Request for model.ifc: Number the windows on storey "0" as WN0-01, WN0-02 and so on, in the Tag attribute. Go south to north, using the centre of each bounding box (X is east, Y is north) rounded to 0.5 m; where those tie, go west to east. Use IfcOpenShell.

First a look at what the model holds.

```python
import ifcopenshell
import ifcopenshell.util.element
import ifcopenshell.util.placement

model = ifcopenshell.open("model.ifc")
print(model.schema)
storey = next(s for s in model.by_type("IfcBuildingStorey") if s.Name == "0")
windows = [e for e in ifcopenshell.util.element.get_decomposition(storey) if e.is_a("IfcWindow")]
for e in sorted(windows, key=lambda e: e.id()):
    origin = ifcopenshell.util.placement.get_local_placement(e.ObjectPlacement)[:3, 3]
    print(e.id(), e.Tag, e.Name, origin.round(2) + 0.0, sep=" | ")
```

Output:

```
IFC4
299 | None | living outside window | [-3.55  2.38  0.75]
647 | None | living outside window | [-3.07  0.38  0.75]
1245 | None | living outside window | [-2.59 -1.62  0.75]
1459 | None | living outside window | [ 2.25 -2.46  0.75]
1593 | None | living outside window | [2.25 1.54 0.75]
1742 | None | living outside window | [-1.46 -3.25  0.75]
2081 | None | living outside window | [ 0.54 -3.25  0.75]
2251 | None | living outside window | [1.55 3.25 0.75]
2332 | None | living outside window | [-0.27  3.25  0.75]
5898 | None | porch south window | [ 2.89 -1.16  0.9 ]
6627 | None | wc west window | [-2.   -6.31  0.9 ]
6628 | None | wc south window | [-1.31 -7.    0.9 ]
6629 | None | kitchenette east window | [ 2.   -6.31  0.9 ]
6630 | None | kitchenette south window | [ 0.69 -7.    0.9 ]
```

```python
import ifcopenshell
import ifcopenshell.geom
import ifcopenshell.util.element
import ifcopenshell.util.shape

model = ifcopenshell.open("model.ifc")
settings = ifcopenshell.geom.settings()
settings.set("use-world-coords", True)


def centre(element):
    shape = ifcopenshell.geom.create_shape(settings, element)
    return ifcopenshell.util.shape.get_bbox_centroid(shape.geometry)


storey = next(s for s in model.by_type("IfcBuildingStorey") if s.Name == "0")
windows = [e for e in ifcopenshell.util.element.get_decomposition(storey) if e.is_a("IfcWindow")]

# Insertion points can sit at a corner or the storey origin, so sort by the geometry (in metres).
centres = {e: centre(e) for e in windows}
windows.sort(key=lambda e: (round(centres[e][1] / 0.5), centres[e][0]))

for i, e in enumerate(windows, start=1):
    number = f"WN0-{i:02d}"
    e.Tag = number
    print(e.id(), number)

model.write("model_edited.ifc")
```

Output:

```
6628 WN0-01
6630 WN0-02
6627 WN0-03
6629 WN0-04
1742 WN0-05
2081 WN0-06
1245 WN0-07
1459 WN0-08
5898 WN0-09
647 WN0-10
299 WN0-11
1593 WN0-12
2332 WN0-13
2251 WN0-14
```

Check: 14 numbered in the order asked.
